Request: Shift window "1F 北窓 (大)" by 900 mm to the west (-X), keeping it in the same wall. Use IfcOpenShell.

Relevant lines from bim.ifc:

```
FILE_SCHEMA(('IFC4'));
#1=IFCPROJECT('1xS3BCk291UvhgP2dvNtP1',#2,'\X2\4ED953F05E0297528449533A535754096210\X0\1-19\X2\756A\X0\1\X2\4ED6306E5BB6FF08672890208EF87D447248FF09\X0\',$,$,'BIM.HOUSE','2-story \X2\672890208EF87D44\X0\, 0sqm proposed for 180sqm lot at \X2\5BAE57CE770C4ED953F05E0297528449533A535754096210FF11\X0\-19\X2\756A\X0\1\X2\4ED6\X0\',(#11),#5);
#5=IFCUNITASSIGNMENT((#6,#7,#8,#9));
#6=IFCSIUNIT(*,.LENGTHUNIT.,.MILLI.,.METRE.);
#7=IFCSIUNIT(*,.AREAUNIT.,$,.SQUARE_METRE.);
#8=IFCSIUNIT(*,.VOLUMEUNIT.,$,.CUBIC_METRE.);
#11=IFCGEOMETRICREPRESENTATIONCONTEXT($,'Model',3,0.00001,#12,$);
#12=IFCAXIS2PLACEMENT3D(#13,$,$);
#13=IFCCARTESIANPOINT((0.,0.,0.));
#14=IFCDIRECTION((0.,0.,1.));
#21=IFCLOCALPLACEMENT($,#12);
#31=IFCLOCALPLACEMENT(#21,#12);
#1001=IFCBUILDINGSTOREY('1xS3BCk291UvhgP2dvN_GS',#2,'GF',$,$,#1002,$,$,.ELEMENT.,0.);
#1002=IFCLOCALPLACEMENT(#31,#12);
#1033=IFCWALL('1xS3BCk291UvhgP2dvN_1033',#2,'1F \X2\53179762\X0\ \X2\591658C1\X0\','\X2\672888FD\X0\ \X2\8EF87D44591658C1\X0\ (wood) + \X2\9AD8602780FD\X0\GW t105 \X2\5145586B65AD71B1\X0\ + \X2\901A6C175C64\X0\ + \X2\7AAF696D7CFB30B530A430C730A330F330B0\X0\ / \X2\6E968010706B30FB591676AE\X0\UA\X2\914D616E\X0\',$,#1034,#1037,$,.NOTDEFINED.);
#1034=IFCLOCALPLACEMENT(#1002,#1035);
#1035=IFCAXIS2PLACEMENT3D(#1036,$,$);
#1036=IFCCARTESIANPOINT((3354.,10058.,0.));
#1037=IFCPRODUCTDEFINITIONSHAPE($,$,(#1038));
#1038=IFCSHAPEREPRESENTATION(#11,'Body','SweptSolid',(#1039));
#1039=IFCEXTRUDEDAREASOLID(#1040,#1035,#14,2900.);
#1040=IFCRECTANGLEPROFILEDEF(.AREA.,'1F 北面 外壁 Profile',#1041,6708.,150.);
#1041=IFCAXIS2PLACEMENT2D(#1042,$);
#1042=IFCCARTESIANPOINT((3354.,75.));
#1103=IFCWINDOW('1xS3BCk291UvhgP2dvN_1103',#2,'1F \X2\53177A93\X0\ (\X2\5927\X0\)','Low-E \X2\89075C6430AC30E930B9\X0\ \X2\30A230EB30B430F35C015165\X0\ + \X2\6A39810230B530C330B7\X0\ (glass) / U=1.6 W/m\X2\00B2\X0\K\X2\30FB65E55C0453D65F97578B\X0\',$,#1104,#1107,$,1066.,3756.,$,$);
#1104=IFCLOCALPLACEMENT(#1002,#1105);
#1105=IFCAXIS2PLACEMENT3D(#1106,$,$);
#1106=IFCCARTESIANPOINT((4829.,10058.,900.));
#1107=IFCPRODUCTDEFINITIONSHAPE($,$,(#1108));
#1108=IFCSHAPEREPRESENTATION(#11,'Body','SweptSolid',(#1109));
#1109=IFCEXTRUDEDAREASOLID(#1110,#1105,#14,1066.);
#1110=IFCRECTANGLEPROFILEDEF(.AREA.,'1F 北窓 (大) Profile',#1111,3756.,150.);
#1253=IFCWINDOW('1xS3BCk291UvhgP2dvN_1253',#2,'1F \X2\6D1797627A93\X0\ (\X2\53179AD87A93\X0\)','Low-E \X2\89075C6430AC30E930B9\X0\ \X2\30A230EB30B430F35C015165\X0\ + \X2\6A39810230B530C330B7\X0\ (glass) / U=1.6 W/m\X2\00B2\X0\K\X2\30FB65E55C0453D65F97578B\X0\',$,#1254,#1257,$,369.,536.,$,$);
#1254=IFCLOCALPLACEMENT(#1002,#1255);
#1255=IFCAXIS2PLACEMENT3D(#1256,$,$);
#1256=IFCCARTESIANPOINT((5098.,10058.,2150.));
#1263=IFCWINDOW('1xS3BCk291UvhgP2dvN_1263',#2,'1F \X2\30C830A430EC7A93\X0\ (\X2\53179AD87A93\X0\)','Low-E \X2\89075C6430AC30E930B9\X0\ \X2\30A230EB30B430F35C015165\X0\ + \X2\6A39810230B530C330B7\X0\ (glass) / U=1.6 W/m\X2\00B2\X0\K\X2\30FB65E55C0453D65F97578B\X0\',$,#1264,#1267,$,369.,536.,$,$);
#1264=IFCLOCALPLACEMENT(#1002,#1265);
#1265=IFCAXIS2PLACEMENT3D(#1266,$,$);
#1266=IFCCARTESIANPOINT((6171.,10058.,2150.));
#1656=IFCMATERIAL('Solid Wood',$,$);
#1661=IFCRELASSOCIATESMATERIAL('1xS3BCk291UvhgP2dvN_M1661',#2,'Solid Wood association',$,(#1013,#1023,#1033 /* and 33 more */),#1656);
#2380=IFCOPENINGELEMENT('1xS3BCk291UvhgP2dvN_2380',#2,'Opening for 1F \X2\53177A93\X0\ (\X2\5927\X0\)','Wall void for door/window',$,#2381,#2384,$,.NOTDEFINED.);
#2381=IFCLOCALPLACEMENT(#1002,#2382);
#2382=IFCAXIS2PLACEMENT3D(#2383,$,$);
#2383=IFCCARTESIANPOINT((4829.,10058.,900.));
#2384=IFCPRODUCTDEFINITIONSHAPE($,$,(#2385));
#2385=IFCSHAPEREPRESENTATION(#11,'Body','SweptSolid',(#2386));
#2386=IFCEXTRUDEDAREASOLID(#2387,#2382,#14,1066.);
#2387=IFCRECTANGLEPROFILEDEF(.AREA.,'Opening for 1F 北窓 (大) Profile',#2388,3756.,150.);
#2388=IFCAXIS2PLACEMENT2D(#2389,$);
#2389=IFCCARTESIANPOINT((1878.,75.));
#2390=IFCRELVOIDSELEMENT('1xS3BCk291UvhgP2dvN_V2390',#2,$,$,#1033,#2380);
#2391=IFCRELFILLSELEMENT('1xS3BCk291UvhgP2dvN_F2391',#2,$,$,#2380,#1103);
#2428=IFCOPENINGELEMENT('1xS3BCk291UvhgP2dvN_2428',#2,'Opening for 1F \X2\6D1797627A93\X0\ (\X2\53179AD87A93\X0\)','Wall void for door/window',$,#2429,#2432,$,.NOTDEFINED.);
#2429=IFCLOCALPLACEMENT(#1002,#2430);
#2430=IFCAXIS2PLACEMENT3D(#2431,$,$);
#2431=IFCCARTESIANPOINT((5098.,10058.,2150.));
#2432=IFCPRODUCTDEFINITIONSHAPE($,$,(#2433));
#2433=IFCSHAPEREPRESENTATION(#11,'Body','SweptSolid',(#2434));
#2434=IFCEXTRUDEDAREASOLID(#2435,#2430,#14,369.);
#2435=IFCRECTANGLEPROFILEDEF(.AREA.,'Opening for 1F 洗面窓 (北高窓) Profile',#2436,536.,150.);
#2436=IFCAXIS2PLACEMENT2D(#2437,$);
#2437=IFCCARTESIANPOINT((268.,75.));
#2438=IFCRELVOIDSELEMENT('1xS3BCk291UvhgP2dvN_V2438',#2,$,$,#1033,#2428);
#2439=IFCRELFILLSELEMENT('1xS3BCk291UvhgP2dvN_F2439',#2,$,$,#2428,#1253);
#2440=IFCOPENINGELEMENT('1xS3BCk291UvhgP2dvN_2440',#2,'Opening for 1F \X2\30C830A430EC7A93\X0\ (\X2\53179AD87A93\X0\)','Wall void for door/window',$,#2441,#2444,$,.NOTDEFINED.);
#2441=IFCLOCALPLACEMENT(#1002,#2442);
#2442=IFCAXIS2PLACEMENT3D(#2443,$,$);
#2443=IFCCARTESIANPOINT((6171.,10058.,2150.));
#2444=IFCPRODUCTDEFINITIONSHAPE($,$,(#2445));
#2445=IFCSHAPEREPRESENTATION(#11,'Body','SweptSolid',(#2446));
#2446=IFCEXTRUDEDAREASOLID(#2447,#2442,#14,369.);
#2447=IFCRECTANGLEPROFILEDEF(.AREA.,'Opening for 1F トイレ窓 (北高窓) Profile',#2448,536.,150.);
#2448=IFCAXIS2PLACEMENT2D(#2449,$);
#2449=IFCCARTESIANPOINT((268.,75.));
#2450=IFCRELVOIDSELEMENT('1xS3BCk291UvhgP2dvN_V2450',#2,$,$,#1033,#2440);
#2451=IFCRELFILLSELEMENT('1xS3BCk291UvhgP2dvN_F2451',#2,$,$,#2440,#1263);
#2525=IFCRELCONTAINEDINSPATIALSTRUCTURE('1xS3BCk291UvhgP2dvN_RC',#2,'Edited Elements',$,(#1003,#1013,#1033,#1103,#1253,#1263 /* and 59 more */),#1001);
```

```python
import ifcopenshell
import ifcopenshell.api.geometry
import ifcopenshell.util.placement

model = ifcopenshell.open("bim.ifc")

window = model.by_guid("1xS3BCk291UvhgP2dvN_1103")
opening = window.FillsVoids[0].RelatingOpeningElement
wall = opening.VoidsElements[0].RelatingBuildingElement

wall_matrix = ifcopenshell.util.placement.get_local_placement(wall.ObjectPlacement)
shift = wall_matrix[:3, 0] * -900.0
before = ifcopenshell.util.placement.get_local_placement(window.ObjectPlacement)[:3, 3].copy()

# The window is not placed relative to its opening, so move both.
for product in (opening, window):
    matrix = ifcopenshell.util.placement.get_local_placement(product.ObjectPlacement)
    matrix[:3, 3] += shift
    ifcopenshell.api.geometry.edit_object_placement(model, product=product, matrix=matrix, is_si=False)

after = ifcopenshell.util.placement.get_local_placement(window.ObjectPlacement)[:3, 3]
print("window moved by", (after - before).round(3) + 0.0)

model.write("bim-out.ifc")
```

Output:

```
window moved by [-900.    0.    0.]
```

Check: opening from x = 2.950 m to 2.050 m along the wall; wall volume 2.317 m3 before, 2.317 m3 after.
